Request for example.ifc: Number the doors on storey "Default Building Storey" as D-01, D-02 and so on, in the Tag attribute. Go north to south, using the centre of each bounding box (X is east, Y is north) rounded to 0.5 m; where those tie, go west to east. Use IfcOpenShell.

First a look at what the model holds.

```python
import ifcopenshell
import ifcopenshell.util.element
import ifcopenshell.util.placement

model = ifcopenshell.open("example.ifc")
print(model.schema)
storey = next(s for s in model.by_type("IfcBuildingStorey") if s.Name == "Default Building Storey")
doors = [e for e in ifcopenshell.util.element.get_decomposition(storey) if e.is_a("IfcDoor")]
for e in sorted(doors, key=lambda e: e.id()):
    origin = ifcopenshell.util.placement.get_local_placement(e.ObjectPlacement)[:3, 3]
    print(e.id(), e.Tag, e.Name, origin.round(2) + 0.0, sep=" | ")
```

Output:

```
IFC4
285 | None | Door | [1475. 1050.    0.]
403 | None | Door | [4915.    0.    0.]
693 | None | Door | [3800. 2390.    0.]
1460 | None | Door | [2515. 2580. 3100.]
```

```python
import ifcopenshell
import ifcopenshell.geom
import ifcopenshell.util.element
import ifcopenshell.util.shape

model = ifcopenshell.open("example.ifc")
settings = ifcopenshell.geom.settings()
settings.set("use-world-coords", True)


def centre(element):
    shape = ifcopenshell.geom.create_shape(settings, element)
    return ifcopenshell.util.shape.get_bbox_centroid(shape.geometry)


storey = next(s for s in model.by_type("IfcBuildingStorey") if s.Name == "Default Building Storey")
doors = [e for e in ifcopenshell.util.element.get_decomposition(storey) if e.is_a("IfcDoor")]

# Insertion points can sit at a corner or the storey origin, so sort by the geometry (in metres).
centres = {e: centre(e) for e in doors}
doors.sort(key=lambda e: (-round(centres[e][1] / 0.5), centres[e][0]))

for i, e in enumerate(doors, start=1):
    number = f"D-{i:02d}"
    e.Tag = number
    print(e.id(), number)

model.write("example_edited.ifc")
```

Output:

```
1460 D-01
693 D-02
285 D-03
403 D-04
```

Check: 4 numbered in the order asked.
